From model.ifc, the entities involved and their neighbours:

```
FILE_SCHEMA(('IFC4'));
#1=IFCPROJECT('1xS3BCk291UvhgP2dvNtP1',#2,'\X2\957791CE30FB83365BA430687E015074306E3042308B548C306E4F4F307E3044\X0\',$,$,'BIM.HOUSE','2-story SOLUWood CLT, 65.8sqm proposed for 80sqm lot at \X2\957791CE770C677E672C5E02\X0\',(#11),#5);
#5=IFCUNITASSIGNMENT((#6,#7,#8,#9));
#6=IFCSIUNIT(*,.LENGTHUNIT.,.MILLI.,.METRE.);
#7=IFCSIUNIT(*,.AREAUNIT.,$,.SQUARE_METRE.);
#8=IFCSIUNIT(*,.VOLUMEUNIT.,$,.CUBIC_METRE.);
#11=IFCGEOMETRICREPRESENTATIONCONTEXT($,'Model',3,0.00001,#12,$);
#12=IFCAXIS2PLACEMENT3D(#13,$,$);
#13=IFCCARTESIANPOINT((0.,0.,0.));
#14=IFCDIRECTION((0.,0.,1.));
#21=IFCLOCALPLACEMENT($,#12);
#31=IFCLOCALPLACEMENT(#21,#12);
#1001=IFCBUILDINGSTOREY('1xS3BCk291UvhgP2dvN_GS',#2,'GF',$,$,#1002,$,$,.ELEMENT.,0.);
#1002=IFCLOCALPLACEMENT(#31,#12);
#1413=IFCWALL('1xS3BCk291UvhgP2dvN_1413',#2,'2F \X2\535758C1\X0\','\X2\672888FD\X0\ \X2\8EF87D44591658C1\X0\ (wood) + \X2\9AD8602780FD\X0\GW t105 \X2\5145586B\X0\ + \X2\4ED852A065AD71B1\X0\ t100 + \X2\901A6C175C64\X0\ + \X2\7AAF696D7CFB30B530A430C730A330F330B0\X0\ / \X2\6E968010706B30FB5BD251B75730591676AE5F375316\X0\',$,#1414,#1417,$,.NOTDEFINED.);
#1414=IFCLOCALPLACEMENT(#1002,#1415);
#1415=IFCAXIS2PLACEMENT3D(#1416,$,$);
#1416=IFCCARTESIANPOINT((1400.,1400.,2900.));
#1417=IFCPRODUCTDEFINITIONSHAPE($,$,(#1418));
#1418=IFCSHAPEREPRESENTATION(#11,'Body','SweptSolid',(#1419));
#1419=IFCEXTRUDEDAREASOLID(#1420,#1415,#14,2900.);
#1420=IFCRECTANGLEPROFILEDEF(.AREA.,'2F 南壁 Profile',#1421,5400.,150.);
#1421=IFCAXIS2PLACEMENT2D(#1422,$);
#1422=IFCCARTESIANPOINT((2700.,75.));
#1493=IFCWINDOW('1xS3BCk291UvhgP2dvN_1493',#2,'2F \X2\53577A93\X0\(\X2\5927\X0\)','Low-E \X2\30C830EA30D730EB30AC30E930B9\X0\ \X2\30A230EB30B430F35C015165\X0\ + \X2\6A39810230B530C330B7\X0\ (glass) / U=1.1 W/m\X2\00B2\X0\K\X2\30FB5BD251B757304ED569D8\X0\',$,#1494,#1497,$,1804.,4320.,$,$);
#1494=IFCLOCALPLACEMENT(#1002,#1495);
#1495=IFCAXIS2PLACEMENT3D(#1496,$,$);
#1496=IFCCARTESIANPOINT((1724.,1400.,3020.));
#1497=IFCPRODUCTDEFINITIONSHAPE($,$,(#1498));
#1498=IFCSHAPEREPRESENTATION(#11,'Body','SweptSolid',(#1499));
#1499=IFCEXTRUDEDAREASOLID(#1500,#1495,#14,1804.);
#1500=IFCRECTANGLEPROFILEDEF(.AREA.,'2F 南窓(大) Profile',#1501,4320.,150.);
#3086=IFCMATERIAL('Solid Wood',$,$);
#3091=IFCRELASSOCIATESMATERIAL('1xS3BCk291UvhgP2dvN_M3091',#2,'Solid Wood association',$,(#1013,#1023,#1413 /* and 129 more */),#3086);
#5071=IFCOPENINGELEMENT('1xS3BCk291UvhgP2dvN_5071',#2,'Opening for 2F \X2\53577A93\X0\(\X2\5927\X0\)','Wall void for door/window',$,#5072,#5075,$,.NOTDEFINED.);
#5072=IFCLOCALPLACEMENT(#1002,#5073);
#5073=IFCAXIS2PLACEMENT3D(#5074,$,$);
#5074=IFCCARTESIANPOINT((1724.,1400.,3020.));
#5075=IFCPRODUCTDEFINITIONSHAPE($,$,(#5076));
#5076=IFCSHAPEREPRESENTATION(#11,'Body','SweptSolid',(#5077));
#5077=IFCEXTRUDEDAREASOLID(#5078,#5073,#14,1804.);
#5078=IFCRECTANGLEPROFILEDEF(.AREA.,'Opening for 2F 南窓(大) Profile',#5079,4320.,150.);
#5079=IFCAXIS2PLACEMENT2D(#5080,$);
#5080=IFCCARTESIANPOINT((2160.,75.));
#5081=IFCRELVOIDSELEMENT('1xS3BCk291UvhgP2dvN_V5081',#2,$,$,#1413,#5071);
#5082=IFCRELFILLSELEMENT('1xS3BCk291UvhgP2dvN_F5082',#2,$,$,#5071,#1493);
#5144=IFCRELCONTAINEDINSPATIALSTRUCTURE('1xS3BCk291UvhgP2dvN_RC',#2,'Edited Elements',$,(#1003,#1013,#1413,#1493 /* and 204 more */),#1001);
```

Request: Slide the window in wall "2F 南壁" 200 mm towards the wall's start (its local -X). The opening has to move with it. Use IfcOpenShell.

```python
import ifcopenshell
import ifcopenshell.api.geometry
import ifcopenshell.util.placement

model = ifcopenshell.open("model.ifc")

window = model.by_id(1493)
opening = window.FillsVoids[0].RelatingOpeningElement
wall = opening.VoidsElements[0].RelatingBuildingElement

wall_matrix = ifcopenshell.util.placement.get_local_placement(wall.ObjectPlacement)
shift = wall_matrix[:3, 0] * -200.0
before = ifcopenshell.util.placement.get_local_placement(window.ObjectPlacement)[:3, 3].copy()

# The window is not placed relative to its opening, so move both.
for product in (opening, window):
    matrix = ifcopenshell.util.placement.get_local_placement(product.ObjectPlacement)
    matrix[:3, 3] += shift
    ifcopenshell.api.geometry.edit_object_placement(model, product=product, matrix=matrix, is_si=False)

after = ifcopenshell.util.placement.get_local_placement(window.ObjectPlacement)[:3, 3]
print("window moved by", (after - before).round(3) + 0.0)

model.write("model_updated.ifc")
```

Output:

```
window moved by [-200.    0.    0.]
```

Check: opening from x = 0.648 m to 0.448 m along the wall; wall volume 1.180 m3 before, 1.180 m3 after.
